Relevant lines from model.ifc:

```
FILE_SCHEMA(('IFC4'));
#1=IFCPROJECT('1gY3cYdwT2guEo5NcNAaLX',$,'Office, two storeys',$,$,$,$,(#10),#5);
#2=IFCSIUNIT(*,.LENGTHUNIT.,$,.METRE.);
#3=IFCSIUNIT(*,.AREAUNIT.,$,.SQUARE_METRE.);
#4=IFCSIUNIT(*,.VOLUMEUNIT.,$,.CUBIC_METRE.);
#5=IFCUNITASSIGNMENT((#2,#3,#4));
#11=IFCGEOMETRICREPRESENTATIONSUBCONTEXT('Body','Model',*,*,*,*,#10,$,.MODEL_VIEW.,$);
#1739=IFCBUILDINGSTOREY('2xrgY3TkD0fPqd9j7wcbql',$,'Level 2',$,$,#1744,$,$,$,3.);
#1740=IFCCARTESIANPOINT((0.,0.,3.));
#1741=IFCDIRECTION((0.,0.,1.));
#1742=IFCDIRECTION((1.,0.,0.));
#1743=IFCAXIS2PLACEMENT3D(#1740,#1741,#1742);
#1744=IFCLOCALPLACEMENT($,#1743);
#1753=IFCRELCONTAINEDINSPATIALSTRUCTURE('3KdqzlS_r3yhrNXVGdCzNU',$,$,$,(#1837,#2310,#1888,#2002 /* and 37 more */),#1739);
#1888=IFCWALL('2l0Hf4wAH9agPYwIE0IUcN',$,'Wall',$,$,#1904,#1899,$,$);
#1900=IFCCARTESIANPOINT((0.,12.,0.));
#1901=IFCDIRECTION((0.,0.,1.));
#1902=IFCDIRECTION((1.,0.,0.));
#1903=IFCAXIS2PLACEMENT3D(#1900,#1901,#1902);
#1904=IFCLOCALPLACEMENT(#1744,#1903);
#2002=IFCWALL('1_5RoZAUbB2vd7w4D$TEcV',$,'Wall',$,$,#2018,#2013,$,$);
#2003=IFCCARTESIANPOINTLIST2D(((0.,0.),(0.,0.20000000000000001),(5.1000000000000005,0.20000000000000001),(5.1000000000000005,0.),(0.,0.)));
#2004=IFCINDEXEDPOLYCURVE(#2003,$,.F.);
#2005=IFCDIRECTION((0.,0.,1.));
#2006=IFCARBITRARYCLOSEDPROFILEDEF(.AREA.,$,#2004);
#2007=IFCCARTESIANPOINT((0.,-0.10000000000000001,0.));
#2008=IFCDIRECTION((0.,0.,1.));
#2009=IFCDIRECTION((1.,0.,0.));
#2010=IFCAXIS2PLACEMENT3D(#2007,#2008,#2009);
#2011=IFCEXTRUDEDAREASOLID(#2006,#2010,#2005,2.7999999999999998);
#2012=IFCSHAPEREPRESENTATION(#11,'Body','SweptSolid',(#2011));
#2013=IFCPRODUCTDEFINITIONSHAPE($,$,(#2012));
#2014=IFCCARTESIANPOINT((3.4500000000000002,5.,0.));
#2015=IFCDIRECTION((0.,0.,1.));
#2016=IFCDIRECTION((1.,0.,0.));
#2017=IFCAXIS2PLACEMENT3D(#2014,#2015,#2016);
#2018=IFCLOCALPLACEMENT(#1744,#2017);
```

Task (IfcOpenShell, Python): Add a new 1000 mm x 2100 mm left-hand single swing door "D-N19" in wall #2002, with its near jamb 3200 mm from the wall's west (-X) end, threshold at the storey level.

```python
import numpy as np
import ifcopenshell
import ifcopenshell.api.feature
import ifcopenshell.api.geometry
import ifcopenshell.api.root
import ifcopenshell.api.spatial
import ifcopenshell.geom
import ifcopenshell.util.element
import ifcopenshell.util.placement
import ifcopenshell.util.representation
import ifcopenshell.util.shape
import ifcopenshell.util.unit

model = ifcopenshell.open("model.ifc")
unit_scale = ifcopenshell.util.unit.calculate_unit_scale(model)
settings = ifcopenshell.geom.settings()


def volume(element):
    """Net volume in cubic metres, openings subtracted."""
    shape = ifcopenshell.geom.create_shape(settings, element)
    return ifcopenshell.util.shape.get_volume(shape.geometry)


wall = model.by_id(2002)
storey = ifcopenshell.util.element.get_container(wall, ifc_class="IfcBuildingStorey")
context = ifcopenshell.util.representation.get_context(model, "Model", "Body", "MODEL_VIEW")
before = volume(wall)

width, height, from_end, sill = 1, 2.1, 3.2, 0.0  # metres

# The wall runs along its own X axis, and the end named is its -X end.
wall_shape = ifcopenshell.geom.create_shape(settings, wall)
x, y, z = ifcopenshell.util.shape.get_vertices(wall_shape.geometry).T
start = x.min() + from_end
face, thickness = float(y.min()), float(y.max() - y.min())
wall_matrix = ifcopenshell.util.placement.get_local_placement(wall.ObjectPlacement)
level = ifcopenshell.util.placement.get_local_placement(storey.ObjectPlacement)[2, 3]


def in_wall(x, y):
    """Placement at x, y metres in the wall's axes, at sill height."""
    matrix = wall_matrix.copy()
    matrix[:, 3] = wall_matrix @ np.array([x / unit_scale, y / unit_scale, 0.0, 1.0])
    matrix[2, 3] = level + sill / unit_scale
    return matrix


# Opening: a box that overshoots both wall faces by 50 mm.
opening = ifcopenshell.api.root.create_entity(model, ifc_class="IfcOpeningElement", predefined_type="OPENING")
box = ifcopenshell.api.geometry.add_wall_representation(
    model, context=context, length=width, height=height, thickness=thickness + 0.1
)
ifcopenshell.api.geometry.assign_representation(model, product=opening, representation=box)
ifcopenshell.api.geometry.edit_object_placement(model, product=opening, matrix=in_wall(start, face - 0.05), is_si=False)
ifcopenshell.api.feature.add_feature(model, feature=opening, element=wall)

door = ifcopenshell.api.root.create_entity(model, ifc_class="IfcDoor", name="D-N19", predefined_type="DOOR")
door.OverallWidth, door.OverallHeight = width / unit_scale, height / unit_scale
door.OperationType = "SINGLE_SWING_LEFT"
body = ifcopenshell.api.geometry.add_door_representation(
    model,
    context=context,
    overall_width=door.OverallWidth,
    overall_height=door.OverallHeight,
    operation_type="SINGLE_SWING_LEFT",
    lining_properties={"LiningDepth": thickness / unit_scale, "ThresholdDepth": thickness / unit_scale},
)
ifcopenshell.api.geometry.assign_representation(model, product=door, representation=body)
ifcopenshell.api.spatial.assign_container(model, products=[door], relating_structure=storey)
ifcopenshell.api.feature.add_filling(model, opening=opening, element=door)

# The lining spans the wall, so the door starts at the wall face.
ifcopenshell.api.geometry.edit_object_placement(model, product=door, matrix=in_wall(start, face), is_si=False)

after = volume(wall)

print(f"wall volume {before:.3f} -> {after:.3f} m3")

model.write("model_updated.ifc")
```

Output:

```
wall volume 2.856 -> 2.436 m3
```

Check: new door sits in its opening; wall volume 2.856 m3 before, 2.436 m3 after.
